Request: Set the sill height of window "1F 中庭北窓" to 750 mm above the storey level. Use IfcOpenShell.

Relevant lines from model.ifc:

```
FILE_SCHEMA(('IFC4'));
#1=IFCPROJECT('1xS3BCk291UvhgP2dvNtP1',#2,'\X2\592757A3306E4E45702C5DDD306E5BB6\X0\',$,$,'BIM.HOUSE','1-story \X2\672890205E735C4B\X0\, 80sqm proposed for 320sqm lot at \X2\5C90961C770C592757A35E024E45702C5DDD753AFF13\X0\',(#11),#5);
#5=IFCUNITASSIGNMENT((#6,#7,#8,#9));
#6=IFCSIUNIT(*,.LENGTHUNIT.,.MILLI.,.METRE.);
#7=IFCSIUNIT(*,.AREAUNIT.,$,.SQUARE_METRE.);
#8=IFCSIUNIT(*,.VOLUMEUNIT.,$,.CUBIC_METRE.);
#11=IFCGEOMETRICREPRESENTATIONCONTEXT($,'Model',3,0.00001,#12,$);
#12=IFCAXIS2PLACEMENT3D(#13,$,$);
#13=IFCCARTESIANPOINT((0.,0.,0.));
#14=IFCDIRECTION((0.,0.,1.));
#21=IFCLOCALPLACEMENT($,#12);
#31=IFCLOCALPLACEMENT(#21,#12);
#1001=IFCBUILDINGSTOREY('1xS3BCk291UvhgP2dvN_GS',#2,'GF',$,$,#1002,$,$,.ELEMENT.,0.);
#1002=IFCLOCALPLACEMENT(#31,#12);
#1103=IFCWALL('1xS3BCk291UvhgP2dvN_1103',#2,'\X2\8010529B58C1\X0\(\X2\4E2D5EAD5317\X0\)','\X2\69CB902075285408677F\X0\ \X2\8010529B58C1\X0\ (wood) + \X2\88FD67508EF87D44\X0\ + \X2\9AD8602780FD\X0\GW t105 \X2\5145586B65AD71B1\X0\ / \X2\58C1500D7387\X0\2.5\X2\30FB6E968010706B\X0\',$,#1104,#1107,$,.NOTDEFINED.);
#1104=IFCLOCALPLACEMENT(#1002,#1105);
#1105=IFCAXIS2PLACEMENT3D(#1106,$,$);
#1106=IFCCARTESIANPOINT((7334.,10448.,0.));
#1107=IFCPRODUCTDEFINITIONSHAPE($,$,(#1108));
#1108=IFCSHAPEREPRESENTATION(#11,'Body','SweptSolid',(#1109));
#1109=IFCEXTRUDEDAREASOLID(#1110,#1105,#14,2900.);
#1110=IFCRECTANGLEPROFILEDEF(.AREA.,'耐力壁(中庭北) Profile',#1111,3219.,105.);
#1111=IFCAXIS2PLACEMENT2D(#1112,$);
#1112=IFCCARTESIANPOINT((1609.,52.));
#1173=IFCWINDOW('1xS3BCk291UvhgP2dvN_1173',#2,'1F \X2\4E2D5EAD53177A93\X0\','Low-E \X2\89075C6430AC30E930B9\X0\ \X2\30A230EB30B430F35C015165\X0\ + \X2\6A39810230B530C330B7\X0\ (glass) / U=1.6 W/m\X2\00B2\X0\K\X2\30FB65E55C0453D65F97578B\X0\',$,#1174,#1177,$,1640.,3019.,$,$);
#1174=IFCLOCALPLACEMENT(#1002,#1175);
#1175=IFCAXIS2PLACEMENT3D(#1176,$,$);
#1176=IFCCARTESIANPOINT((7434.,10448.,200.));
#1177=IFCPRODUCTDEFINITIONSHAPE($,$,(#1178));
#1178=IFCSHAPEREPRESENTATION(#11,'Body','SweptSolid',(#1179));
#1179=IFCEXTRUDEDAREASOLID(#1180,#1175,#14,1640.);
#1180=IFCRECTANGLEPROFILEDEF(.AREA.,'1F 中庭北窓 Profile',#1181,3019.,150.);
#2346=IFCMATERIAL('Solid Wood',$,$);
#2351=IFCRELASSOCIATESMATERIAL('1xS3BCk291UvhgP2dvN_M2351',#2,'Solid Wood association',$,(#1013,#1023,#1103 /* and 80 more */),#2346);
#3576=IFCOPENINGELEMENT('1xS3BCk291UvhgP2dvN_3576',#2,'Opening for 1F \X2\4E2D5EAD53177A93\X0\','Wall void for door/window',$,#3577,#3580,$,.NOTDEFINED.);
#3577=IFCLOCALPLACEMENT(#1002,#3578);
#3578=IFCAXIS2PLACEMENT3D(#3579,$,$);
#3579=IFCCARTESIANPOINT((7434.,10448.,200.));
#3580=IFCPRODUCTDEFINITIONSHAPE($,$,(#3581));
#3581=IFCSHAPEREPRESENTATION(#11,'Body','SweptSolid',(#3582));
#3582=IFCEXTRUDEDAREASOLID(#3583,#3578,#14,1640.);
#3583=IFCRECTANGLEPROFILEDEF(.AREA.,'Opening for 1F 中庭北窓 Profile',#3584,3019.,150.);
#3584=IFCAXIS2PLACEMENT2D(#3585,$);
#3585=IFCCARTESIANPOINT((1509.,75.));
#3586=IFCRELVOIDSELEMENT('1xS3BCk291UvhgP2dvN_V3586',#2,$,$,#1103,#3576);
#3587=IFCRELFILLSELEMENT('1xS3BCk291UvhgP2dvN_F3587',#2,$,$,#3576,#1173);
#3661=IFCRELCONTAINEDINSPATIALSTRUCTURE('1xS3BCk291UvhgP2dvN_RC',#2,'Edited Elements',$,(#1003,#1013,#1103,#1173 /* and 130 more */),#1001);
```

```python
import numpy as np
import ifcopenshell
import ifcopenshell.api.geometry
import ifcopenshell.geom
import ifcopenshell.util.element
import ifcopenshell.util.placement
import ifcopenshell.util.shape
import ifcopenshell.util.unit

model = ifcopenshell.open("model.ifc")
unit_scale = ifcopenshell.util.unit.calculate_unit_scale(model)

window = model.by_guid("1xS3BCk291UvhgP2dvN_1173")
opening = window.FillsVoids[0].RelatingOpeningElement
storey = ifcopenshell.util.element.get_container(window, ifc_class="IfcBuildingStorey")
level = ifcopenshell.util.placement.get_local_placement(storey.ObjectPlacement)[2, 3]

# The opening's origin need not be at the sill, so measure its lowest point.
shape = ifcopenshell.geom.create_shape(ifcopenshell.geom.settings(), opening)
bottom = ifcopenshell.util.shape.get_shape_bottom_elevation(shape, shape.geometry) / unit_scale
dz = level + 0.75 / unit_scale - bottom

shift = np.array([0.0, 0.0, dz])
# The window is not placed relative to its opening, so move both.
for product in (opening, window):
    matrix = ifcopenshell.util.placement.get_local_placement(product.ObjectPlacement)
    matrix[:3, 3] += shift
    ifcopenshell.api.geometry.edit_object_placement(model, product=product, matrix=matrix, is_si=False)

print(f"moved by {dz * unit_scale:+.3f} m")

model.write("model_rev.ifc")
```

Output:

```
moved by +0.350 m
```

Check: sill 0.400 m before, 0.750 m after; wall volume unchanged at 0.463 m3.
